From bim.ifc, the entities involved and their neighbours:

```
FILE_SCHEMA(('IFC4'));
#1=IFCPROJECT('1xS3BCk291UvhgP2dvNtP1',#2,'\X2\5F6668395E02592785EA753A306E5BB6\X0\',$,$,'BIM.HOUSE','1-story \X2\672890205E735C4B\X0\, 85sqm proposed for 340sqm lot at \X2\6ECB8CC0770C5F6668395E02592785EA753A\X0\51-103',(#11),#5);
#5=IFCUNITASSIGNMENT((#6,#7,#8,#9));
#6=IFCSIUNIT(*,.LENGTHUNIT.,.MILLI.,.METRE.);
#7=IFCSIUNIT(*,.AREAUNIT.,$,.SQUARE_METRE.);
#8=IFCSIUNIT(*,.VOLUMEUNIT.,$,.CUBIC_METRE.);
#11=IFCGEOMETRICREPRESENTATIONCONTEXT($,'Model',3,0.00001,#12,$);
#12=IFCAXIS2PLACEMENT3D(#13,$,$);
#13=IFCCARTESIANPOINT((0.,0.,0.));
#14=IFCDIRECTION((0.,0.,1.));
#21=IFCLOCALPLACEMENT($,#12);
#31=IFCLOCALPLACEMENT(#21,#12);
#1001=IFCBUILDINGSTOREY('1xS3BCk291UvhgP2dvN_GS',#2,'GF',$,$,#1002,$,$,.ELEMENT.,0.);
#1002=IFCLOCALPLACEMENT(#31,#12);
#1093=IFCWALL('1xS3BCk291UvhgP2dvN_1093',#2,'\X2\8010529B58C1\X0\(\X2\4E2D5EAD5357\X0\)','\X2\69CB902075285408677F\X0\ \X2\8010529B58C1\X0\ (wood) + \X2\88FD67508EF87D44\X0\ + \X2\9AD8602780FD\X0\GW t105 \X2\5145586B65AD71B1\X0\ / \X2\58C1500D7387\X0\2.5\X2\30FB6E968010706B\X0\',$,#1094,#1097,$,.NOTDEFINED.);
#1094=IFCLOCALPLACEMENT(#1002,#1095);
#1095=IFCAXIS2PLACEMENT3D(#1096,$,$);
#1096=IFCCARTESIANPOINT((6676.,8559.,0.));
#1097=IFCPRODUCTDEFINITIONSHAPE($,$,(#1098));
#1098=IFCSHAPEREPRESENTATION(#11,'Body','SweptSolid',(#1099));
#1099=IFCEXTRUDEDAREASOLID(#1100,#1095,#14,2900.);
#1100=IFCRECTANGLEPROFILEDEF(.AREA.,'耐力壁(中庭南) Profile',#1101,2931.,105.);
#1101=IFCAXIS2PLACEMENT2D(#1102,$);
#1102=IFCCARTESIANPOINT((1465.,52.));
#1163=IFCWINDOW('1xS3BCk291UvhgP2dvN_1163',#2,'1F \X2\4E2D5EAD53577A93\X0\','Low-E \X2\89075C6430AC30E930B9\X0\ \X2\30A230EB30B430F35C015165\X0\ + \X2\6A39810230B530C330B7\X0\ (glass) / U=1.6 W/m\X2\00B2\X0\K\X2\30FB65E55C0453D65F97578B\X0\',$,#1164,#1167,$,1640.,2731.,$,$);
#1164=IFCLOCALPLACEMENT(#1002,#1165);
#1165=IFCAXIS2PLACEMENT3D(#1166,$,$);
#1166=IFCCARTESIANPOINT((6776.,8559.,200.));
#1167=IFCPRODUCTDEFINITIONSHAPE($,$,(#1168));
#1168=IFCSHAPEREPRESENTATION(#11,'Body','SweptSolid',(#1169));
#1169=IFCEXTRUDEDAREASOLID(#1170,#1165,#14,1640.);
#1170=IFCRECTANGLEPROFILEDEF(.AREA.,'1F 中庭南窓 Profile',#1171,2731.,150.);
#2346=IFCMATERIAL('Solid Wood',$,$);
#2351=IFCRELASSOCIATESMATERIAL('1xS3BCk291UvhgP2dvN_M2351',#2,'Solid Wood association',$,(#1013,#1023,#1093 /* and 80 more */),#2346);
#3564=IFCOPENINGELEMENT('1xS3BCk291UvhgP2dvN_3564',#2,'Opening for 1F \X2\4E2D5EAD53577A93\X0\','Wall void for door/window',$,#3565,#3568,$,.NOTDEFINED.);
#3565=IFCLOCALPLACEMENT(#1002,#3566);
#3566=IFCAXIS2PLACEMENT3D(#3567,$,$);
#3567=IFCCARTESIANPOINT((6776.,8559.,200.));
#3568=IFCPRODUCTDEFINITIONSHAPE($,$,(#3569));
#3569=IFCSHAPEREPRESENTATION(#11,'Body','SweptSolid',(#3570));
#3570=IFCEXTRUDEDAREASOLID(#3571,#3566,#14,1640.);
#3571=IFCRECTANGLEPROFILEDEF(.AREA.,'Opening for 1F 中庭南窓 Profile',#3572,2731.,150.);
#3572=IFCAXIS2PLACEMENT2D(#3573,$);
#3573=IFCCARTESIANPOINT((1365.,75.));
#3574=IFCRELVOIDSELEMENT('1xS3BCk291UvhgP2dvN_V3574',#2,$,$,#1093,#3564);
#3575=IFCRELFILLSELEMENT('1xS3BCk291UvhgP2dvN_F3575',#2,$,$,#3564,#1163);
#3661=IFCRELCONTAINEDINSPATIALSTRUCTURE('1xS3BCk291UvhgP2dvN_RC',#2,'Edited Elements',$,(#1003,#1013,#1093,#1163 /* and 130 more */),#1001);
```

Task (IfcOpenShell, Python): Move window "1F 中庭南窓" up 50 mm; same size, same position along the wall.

```python
import numpy as np
import ifcopenshell
import ifcopenshell.api.geometry
import ifcopenshell.util.placement
import ifcopenshell.util.unit

model = ifcopenshell.open("bim.ifc")
unit_scale = ifcopenshell.util.unit.calculate_unit_scale(model)

window = model.by_guid("1xS3BCk291UvhgP2dvN_1163")
opening = window.FillsVoids[0].RelatingOpeningElement
dz = 50.0

shift = np.array([0.0, 0.0, dz])
# The window is not placed relative to its opening, so move both.
for product in (opening, window):
    matrix = ifcopenshell.util.placement.get_local_placement(product.ObjectPlacement)
    matrix[:3, 3] += shift
    ifcopenshell.api.geometry.edit_object_placement(model, product=product, matrix=matrix, is_si=False)

print(f"moved by {dz * unit_scale:+.3f} m")

model.write("bim_v2.ifc")
```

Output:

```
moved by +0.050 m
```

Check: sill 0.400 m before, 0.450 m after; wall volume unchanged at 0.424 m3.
